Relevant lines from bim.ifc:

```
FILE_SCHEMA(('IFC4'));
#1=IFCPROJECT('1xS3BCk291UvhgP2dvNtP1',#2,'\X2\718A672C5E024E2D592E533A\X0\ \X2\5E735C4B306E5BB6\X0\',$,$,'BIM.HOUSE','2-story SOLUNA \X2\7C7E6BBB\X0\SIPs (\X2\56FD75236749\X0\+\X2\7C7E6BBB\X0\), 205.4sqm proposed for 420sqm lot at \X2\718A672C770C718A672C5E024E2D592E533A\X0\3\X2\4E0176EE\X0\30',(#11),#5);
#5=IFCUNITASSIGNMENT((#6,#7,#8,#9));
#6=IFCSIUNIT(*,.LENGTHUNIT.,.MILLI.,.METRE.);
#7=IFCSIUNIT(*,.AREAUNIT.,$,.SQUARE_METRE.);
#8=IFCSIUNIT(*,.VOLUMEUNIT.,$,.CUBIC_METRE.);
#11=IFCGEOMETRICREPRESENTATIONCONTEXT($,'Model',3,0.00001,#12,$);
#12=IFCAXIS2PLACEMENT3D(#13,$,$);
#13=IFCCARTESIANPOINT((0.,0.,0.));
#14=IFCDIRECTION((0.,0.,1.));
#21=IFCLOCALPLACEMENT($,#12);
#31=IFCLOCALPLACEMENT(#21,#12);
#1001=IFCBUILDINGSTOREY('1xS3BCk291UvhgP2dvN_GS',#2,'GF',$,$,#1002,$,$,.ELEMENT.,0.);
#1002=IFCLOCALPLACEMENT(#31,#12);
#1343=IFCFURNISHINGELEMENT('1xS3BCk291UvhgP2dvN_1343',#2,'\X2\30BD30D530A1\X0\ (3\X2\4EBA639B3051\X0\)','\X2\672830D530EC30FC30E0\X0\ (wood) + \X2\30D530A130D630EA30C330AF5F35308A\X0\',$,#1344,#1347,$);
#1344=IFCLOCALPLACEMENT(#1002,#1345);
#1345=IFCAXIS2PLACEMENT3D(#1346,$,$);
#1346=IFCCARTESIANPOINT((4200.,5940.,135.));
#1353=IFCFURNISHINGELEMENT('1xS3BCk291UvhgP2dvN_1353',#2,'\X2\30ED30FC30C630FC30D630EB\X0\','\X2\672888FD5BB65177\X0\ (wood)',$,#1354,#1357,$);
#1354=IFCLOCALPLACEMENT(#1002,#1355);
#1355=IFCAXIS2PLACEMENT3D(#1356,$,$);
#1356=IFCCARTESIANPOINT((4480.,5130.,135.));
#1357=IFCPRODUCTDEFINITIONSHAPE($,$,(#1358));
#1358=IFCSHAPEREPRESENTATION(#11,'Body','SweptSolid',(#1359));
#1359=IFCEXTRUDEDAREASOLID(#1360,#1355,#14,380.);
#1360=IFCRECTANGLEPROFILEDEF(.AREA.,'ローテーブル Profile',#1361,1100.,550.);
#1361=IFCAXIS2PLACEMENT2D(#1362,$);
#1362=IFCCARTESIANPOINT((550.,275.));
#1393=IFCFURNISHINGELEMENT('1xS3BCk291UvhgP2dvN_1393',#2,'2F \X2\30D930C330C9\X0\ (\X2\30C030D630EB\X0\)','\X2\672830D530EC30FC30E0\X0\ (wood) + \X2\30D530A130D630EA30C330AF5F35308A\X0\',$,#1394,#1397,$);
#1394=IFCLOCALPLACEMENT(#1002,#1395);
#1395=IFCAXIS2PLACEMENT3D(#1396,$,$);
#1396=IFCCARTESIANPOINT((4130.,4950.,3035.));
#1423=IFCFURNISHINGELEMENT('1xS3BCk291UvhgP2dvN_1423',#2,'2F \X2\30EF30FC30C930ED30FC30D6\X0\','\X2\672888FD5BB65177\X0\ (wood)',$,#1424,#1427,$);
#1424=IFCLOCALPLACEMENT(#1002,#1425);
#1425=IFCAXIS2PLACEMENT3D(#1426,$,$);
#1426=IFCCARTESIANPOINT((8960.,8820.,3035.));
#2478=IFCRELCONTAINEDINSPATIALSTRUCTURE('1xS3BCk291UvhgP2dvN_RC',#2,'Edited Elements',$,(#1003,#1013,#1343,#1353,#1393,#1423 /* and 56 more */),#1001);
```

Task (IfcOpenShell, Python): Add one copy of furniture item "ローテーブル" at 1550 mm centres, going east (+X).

```python
import numpy as np
import ifcopenshell
import ifcopenshell.api.geometry
import ifcopenshell.api.root
import ifcopenshell.util.element
import ifcopenshell.util.placement
import ifcopenshell.util.unit

model = ifcopenshell.open("bim.ifc")
unit_scale = ifcopenshell.util.unit.calculate_unit_scale(model)


def reuse_history(source, copy):
    """copy_class also copies each property set's owner history, people and application; keep the originals."""
    for rel in copy.IsDefinedBy:
        if rel.is_a("IfcRelDefinesByProperties") and (history := rel.RelatingPropertyDefinition.OwnerHistory):
            rel.RelatingPropertyDefinition.OwnerHistory = source.OwnerHistory
            ifcopenshell.util.element.remove_deep2(model, history)


source = model.by_id(1353)
base = ifcopenshell.util.placement.get_local_placement(source.ObjectPlacement)
step = np.array([1.0, 0.0, 0.0]) * 1.55 / unit_scale

for i in range(1, 2):
    copy = ifcopenshell.api.root.copy_class(model, product=source)
    copy.Representation = ifcopenshell.util.element.copy_deep(
        model, source.Representation, exclude=["IfcGeometricRepresentationContext", "IfcRepresentationMap"]
    )
    reuse_history(source, copy)
    matrix = base.copy()
    matrix[:3, 3] += i * step
    print("added at", matrix[:3, 3].round(3) + 0.0)
    ifcopenshell.api.geometry.edit_object_placement(model, product=copy, matrix=matrix, is_si=False)

model.write("bim_updated.ifc")
```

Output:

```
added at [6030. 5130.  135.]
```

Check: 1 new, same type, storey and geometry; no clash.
